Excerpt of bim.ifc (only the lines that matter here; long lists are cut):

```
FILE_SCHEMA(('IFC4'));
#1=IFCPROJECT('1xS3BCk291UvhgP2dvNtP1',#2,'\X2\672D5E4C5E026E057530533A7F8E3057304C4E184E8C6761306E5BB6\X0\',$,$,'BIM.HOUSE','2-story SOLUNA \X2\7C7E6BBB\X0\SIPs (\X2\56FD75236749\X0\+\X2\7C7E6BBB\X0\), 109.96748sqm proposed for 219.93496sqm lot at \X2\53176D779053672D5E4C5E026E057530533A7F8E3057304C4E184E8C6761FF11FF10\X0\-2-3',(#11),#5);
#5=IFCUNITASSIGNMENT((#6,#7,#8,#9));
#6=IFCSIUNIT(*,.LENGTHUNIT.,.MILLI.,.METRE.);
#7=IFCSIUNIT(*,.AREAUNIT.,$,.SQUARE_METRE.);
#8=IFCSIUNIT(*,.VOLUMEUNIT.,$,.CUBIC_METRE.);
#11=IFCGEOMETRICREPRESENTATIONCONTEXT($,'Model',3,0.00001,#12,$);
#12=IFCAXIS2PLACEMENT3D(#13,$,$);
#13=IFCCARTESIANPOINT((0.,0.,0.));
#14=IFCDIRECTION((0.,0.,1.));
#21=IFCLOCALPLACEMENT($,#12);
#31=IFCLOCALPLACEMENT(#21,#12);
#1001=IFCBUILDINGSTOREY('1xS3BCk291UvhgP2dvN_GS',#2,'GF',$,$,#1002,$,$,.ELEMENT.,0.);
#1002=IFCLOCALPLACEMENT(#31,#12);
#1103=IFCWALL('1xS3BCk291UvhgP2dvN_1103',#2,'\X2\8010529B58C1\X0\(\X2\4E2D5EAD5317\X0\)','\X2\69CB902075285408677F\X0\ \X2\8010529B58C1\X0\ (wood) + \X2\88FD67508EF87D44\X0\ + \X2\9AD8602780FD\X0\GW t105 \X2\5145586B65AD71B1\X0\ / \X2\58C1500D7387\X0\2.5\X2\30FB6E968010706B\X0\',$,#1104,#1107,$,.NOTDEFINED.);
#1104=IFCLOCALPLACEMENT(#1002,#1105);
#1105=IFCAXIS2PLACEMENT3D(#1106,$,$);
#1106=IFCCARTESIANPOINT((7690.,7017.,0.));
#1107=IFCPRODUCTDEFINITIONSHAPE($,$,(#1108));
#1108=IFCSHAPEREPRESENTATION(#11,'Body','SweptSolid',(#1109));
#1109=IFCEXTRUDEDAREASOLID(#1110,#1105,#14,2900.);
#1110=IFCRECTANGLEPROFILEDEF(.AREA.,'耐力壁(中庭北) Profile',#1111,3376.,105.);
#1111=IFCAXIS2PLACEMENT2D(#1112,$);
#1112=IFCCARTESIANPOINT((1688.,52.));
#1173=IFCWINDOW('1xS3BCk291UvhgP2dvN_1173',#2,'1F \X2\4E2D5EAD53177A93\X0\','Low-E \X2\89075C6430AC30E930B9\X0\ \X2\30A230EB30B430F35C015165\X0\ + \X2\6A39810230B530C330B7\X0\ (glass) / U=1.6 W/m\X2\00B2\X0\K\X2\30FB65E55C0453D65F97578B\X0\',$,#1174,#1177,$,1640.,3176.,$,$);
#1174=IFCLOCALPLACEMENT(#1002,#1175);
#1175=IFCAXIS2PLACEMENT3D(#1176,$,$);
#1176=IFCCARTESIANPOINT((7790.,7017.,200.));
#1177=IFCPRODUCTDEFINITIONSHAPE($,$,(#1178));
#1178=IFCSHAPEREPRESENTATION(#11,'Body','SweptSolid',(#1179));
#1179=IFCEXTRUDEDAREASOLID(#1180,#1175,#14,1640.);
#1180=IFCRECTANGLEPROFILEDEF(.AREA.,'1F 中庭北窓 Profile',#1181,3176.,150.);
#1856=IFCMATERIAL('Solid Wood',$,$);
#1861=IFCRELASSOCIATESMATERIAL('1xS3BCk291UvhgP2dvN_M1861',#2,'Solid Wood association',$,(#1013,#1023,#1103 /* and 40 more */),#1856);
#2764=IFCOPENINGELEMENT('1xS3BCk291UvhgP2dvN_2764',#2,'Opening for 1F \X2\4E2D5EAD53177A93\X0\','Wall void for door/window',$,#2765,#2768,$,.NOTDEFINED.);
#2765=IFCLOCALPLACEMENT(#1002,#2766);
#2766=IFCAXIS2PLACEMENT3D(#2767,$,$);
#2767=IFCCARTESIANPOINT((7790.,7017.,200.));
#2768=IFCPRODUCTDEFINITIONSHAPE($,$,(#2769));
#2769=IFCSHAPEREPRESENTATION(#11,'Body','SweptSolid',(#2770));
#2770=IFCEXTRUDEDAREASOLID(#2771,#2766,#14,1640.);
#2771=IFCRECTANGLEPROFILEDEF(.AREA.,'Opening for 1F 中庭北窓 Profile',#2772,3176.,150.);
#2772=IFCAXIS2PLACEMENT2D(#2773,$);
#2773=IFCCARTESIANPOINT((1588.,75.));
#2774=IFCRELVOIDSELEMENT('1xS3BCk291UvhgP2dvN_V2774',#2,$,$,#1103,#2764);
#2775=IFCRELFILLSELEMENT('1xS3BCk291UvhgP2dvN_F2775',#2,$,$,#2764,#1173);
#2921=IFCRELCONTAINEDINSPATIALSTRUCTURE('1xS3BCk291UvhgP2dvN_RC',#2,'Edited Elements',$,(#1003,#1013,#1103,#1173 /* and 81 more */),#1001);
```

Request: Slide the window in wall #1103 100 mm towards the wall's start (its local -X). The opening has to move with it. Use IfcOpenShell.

```python
import ifcopenshell
import ifcopenshell.api.geometry
import ifcopenshell.util.placement
import ifcopenshell.util.unit

model = ifcopenshell.open("bim.ifc")
unit_scale = ifcopenshell.util.unit.calculate_unit_scale(model)

window = model.by_id(1173)
opening = window.FillsVoids[0].RelatingOpeningElement
wall = opening.VoidsElements[0].RelatingBuildingElement

wall_matrix = ifcopenshell.util.placement.get_local_placement(wall.ObjectPlacement)
shift = wall_matrix[:3, 0] * -0.1 / unit_scale
before = ifcopenshell.util.placement.get_local_placement(window.ObjectPlacement)[:3, 3].copy()

# The window is not placed relative to its opening, so move both.
for product in (opening, window):
    matrix = ifcopenshell.util.placement.get_local_placement(product.ObjectPlacement)
    matrix[:3, 3] += shift
    ifcopenshell.api.geometry.edit_object_placement(model, product=product, matrix=matrix, is_si=False)

after = ifcopenshell.util.placement.get_local_placement(window.ObjectPlacement)[:3, 3]
print("window moved by", (after - before).round(3) + 0.0)

model.write("bim_edited.ifc")
```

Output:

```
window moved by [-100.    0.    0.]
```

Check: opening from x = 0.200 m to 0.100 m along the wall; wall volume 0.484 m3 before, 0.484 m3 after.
